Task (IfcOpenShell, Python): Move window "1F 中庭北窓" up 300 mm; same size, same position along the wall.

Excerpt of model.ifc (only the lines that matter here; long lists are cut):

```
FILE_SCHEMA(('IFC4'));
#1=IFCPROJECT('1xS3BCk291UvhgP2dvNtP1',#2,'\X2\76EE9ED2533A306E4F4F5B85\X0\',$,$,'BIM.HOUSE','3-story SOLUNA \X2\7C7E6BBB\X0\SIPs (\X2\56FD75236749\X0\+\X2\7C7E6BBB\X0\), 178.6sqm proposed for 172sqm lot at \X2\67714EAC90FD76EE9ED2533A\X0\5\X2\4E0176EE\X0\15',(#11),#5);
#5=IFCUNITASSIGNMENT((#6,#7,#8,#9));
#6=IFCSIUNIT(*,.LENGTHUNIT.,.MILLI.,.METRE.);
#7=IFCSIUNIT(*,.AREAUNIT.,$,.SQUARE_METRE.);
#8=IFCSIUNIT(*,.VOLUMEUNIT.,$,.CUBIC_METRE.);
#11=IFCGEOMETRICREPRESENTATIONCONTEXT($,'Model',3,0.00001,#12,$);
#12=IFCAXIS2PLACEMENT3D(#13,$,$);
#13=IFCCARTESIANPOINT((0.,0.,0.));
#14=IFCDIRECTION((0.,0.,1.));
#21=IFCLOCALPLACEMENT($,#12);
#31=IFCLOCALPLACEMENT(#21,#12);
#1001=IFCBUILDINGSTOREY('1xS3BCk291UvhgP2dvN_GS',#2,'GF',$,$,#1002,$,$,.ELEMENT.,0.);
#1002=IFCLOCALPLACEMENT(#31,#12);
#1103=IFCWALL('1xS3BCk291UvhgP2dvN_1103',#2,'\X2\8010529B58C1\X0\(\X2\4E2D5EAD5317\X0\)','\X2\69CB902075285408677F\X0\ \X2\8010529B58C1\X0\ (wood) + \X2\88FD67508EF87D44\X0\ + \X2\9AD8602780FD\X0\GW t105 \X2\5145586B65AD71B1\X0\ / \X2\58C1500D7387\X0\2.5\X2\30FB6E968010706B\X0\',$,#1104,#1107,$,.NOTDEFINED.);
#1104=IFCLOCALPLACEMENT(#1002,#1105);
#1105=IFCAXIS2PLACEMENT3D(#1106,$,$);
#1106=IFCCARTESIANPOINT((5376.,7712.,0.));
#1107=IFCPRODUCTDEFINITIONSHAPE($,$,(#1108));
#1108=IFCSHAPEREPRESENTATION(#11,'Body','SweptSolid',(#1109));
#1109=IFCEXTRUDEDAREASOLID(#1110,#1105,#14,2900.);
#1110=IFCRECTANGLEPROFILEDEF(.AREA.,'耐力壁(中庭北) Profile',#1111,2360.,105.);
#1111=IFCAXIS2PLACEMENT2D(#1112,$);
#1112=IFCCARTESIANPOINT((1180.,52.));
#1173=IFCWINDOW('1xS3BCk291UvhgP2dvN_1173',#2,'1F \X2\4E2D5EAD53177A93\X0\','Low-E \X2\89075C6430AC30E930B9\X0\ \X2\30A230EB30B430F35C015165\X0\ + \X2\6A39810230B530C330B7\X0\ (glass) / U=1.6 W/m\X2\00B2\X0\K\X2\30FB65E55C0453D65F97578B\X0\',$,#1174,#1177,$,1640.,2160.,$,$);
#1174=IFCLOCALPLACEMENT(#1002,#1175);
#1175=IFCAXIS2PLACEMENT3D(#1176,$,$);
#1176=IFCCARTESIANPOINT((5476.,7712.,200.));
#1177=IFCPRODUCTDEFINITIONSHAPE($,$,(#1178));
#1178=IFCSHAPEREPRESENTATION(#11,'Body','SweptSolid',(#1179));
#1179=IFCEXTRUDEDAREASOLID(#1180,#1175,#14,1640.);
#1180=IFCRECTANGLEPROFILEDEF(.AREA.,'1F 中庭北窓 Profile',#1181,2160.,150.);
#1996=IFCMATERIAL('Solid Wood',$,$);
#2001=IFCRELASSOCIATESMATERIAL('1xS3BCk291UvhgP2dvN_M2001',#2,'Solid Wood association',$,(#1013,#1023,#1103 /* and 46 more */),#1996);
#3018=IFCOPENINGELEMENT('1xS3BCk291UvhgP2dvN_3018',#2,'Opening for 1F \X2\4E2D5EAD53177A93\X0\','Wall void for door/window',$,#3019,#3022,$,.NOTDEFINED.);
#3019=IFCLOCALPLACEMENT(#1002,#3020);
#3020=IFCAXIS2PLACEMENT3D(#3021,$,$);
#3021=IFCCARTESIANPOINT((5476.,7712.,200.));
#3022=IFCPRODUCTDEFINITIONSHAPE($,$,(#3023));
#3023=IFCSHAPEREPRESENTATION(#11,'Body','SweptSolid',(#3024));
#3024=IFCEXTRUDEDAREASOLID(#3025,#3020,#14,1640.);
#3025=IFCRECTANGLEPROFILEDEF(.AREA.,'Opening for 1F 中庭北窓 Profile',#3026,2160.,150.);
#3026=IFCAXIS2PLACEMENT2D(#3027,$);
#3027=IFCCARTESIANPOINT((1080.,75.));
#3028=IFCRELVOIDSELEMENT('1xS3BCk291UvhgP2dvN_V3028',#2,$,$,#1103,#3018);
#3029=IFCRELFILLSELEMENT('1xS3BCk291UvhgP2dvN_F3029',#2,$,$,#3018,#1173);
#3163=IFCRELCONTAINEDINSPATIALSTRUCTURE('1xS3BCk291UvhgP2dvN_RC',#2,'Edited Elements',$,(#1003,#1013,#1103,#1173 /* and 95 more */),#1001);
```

```python
import numpy as np
import ifcopenshell
import ifcopenshell.api.geometry
import ifcopenshell.util.placement
import ifcopenshell.util.unit

model = ifcopenshell.open("model.ifc")
unit_scale = ifcopenshell.util.unit.calculate_unit_scale(model)

window = model.by_guid("1xS3BCk291UvhgP2dvN_1173")
opening = window.FillsVoids[0].RelatingOpeningElement
dz = 0.3 / unit_scale

shift = np.array([0.0, 0.0, dz])
# The window is not placed relative to its opening, so move both.
for product in (opening, window):
    matrix = ifcopenshell.util.placement.get_local_placement(product.ObjectPlacement)
    matrix[:3, 3] += shift
    ifcopenshell.api.geometry.edit_object_placement(model, product=product, matrix=matrix, is_si=False)

print(f"moved by {dz * unit_scale:+.3f} m")

model.write("model_updated.ifc")
```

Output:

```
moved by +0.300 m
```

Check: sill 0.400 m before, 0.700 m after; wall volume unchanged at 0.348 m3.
